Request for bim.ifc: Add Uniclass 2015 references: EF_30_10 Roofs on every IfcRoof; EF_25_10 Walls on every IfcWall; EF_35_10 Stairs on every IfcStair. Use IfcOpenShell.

First a look at what the model holds.

```python
import ifcopenshell

model = ifcopenshell.open("bim.ifc")
print(model.schema)
print("classifications:", [c.Name for c in model.by_type("IfcClassification")])
for ifc_class in ("IfcDoor", "IfcRoof", "IfcStair", "IfcWall", "IfcWindow"):
    print(ifc_class, len(model.by_type(ifc_class)))
```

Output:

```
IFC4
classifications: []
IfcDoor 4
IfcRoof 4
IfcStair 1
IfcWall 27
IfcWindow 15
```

```python
import ifcopenshell
import ifcopenshell.api.classification

model = ifcopenshell.open("bim.ifc")

system = ifcopenshell.api.classification.add_classification(model, classification="Uniclass 2015")

codes = {
    "IfcRoof": ("EF_30_10", "Roofs"),
    "IfcWall": ("EF_25_10", "Walls"),
    "IfcStair": ("EF_35_10", "Stairs"),
}
for ifc_class, (code, name) in codes.items():
    products = model.by_type(ifc_class)
    ifcopenshell.api.classification.add_reference(
        model, products=products, classification=system, identification=code, name=name
    )
    print(code, len(products))

model.write("bim_edited.ifc")
```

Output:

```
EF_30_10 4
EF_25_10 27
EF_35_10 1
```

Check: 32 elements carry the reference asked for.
